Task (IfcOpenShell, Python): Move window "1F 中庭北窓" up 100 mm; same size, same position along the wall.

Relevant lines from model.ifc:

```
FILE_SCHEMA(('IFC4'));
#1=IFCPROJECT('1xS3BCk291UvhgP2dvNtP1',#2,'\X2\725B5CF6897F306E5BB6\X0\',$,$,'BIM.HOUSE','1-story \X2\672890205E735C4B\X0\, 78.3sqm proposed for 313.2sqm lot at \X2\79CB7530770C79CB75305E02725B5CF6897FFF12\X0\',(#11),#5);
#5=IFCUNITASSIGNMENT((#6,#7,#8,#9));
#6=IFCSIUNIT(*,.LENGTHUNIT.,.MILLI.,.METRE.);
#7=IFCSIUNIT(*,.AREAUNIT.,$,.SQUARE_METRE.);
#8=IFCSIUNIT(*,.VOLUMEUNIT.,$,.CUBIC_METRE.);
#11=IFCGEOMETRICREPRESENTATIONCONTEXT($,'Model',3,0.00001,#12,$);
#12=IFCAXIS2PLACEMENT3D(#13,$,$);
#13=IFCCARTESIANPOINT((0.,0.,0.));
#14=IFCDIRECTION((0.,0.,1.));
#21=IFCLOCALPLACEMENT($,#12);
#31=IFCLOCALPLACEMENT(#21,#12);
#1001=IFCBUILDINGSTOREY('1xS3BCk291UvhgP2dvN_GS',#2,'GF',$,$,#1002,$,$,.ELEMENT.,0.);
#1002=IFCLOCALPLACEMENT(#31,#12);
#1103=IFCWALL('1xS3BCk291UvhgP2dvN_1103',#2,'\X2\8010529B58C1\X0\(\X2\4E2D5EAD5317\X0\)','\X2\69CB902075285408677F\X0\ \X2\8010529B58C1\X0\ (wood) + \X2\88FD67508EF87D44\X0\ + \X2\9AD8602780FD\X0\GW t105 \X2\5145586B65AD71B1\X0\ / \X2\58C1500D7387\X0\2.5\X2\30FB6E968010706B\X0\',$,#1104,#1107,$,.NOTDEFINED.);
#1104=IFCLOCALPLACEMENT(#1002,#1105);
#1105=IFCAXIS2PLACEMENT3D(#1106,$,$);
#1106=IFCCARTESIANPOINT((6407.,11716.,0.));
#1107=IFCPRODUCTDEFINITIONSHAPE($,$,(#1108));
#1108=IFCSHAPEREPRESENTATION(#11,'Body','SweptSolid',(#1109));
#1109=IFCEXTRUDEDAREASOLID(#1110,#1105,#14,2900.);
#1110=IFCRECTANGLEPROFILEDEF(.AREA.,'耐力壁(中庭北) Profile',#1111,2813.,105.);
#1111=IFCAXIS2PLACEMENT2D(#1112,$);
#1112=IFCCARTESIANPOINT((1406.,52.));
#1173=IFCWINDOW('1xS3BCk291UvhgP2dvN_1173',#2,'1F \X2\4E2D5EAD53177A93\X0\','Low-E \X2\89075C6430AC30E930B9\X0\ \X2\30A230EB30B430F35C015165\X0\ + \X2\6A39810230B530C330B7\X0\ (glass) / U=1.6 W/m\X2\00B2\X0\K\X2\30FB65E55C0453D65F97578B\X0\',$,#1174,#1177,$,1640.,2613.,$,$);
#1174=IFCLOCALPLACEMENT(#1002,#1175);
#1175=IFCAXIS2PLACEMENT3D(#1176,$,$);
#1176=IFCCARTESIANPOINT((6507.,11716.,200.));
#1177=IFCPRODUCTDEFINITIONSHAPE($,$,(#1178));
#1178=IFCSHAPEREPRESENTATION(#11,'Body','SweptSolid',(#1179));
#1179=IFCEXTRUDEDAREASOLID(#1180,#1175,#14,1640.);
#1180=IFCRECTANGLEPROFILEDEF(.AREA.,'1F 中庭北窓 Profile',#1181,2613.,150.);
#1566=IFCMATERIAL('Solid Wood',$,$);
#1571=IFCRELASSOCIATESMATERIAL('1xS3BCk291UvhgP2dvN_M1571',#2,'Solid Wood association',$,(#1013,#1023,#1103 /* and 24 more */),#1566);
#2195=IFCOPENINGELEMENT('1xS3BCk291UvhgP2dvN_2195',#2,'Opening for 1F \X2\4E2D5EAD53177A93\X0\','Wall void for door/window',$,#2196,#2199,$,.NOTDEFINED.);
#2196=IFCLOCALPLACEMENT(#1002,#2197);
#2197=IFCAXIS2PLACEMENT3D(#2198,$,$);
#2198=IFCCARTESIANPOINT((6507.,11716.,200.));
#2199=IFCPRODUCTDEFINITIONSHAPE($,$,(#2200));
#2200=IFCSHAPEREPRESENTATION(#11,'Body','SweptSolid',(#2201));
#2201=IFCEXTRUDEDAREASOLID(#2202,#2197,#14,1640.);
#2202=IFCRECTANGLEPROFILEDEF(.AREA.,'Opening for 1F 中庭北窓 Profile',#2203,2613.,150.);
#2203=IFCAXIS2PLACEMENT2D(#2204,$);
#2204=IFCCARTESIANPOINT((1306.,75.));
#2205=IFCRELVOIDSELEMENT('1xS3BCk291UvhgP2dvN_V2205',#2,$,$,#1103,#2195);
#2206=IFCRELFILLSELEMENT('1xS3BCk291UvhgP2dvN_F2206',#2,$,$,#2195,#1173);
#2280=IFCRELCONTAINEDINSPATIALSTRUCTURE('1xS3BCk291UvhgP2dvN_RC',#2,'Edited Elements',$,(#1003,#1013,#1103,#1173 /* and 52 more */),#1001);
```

```python
import numpy as np
import ifcopenshell
import ifcopenshell.api.geometry
import ifcopenshell.util.placement
import ifcopenshell.util.unit

model = ifcopenshell.open("model.ifc")
unit_scale = ifcopenshell.util.unit.calculate_unit_scale(model)

window = model.by_guid("1xS3BCk291UvhgP2dvN_1173")
opening = window.FillsVoids[0].RelatingOpeningElement
dz = 100.0

shift = np.array([0.0, 0.0, dz])
# The window is not placed relative to its opening, so move both.
for product in (opening, window):
    matrix = ifcopenshell.util.placement.get_local_placement(product.ObjectPlacement)
    matrix[:3, 3] += shift
    ifcopenshell.api.geometry.edit_object_placement(model, product=product, matrix=matrix, is_si=False)

print(f"moved by {dz * unit_scale:+.3f} m")

model.write("model_updated.ifc")
```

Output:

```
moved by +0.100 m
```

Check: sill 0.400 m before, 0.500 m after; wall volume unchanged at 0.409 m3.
